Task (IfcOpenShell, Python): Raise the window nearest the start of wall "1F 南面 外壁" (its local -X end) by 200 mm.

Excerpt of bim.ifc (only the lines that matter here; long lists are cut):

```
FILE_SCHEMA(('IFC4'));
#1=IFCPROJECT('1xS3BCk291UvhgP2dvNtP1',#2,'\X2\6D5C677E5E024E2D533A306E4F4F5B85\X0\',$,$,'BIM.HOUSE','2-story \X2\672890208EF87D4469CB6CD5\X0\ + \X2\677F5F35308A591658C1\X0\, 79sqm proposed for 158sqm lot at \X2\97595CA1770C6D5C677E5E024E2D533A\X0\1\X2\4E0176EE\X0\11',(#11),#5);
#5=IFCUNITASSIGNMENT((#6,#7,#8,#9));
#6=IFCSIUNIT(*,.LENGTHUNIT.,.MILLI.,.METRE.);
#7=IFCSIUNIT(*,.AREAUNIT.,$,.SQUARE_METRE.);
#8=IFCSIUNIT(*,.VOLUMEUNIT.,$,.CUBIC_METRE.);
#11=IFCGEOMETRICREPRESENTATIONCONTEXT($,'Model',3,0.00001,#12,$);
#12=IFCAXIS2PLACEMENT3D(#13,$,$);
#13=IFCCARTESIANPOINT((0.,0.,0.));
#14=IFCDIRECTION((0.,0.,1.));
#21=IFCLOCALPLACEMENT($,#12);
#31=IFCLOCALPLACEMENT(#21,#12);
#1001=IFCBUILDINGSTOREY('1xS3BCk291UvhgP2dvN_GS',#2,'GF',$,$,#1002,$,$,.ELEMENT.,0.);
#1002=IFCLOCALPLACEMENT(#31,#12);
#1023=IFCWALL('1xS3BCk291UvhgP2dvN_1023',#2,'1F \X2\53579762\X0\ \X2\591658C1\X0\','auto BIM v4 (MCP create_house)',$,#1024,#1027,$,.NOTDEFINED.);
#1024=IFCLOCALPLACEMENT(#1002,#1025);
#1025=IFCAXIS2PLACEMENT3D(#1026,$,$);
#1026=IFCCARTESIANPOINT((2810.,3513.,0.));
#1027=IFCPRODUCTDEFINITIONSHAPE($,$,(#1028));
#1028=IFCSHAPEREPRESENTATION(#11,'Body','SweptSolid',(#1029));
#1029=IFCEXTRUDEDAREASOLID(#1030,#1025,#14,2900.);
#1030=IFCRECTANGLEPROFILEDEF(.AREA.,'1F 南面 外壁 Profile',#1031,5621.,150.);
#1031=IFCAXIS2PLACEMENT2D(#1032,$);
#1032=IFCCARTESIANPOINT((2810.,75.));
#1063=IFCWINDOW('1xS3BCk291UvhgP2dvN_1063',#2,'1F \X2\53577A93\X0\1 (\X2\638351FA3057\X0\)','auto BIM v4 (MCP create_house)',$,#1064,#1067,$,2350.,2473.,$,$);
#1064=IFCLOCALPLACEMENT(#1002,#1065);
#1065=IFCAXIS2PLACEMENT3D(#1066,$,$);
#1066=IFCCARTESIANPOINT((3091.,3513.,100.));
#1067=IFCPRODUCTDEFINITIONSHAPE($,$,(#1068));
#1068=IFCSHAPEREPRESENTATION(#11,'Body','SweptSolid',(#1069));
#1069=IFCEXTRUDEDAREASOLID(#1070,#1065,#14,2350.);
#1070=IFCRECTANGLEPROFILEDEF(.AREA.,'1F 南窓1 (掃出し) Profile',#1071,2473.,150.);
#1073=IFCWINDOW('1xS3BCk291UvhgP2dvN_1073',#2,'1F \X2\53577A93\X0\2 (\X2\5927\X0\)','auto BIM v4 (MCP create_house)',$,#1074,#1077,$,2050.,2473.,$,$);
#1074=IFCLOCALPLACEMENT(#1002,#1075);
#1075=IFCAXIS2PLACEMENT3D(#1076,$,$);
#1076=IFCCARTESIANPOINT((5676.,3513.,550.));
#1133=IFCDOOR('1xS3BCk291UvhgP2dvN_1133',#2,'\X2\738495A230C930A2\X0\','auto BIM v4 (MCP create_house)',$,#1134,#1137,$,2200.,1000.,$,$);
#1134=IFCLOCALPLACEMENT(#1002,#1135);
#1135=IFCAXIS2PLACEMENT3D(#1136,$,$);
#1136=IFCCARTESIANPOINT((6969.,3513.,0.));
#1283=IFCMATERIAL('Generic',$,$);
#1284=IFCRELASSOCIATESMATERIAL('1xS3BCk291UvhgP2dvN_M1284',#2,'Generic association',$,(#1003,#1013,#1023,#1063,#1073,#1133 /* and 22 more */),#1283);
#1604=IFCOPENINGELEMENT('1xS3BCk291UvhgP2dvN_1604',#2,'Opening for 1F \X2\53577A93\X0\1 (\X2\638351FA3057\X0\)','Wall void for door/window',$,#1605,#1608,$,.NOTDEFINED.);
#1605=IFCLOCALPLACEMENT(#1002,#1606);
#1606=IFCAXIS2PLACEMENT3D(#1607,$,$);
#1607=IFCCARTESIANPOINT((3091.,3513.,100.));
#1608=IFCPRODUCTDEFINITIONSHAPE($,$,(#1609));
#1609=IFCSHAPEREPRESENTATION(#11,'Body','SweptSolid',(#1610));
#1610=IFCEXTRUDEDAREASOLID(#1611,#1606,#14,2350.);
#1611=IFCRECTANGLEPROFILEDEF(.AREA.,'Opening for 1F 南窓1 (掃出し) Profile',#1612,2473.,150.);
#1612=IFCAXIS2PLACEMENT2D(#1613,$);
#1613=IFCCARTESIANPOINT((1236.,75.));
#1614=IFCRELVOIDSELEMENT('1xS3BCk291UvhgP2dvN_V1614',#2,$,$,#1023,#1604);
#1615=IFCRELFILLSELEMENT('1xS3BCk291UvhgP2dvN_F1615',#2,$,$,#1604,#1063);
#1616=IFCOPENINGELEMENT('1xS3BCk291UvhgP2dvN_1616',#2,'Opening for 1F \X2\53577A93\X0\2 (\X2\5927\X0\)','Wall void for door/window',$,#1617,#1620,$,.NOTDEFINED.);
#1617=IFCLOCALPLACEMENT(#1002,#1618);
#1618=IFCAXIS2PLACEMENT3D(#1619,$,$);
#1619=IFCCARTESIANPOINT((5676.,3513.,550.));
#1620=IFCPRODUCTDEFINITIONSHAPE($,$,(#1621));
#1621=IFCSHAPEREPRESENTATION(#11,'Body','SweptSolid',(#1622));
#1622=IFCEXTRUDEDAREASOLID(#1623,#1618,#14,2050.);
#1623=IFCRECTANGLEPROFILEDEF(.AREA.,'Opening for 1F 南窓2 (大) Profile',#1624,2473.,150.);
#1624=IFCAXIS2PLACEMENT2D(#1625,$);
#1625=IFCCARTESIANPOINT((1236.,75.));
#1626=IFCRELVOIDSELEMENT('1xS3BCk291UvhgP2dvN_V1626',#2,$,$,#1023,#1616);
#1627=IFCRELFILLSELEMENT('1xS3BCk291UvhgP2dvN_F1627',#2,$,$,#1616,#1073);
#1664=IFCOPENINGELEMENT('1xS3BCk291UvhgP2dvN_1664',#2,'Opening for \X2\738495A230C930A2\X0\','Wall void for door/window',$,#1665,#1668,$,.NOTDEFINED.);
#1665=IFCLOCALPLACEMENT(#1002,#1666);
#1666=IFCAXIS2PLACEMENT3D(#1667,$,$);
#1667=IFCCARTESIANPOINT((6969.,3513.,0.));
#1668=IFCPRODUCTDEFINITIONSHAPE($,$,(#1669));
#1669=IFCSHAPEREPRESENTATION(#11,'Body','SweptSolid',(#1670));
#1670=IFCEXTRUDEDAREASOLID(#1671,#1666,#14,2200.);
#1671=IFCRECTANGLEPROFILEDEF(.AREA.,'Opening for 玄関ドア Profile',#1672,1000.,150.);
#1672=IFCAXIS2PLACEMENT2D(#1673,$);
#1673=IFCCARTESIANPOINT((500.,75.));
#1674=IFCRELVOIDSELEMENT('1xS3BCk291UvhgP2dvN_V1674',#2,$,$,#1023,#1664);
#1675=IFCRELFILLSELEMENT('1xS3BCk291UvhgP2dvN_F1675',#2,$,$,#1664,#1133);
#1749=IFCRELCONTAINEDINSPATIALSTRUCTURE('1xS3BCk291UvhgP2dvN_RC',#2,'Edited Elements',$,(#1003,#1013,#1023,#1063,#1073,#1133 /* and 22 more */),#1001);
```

```python
import numpy as np
import ifcopenshell
import ifcopenshell.api.geometry
import ifcopenshell.util.placement
import ifcopenshell.util.unit

model = ifcopenshell.open("bim.ifc")
unit_scale = ifcopenshell.util.unit.calculate_unit_scale(model)

window = model.by_guid("1xS3BCk291UvhgP2dvN_1063")
opening = window.FillsVoids[0].RelatingOpeningElement
dz = 0.2 / unit_scale

shift = np.array([0.0, 0.0, dz])
# The window is not placed relative to its opening, so move both.
for product in (opening, window):
    matrix = ifcopenshell.util.placement.get_local_placement(product.ObjectPlacement)
    matrix[:3, 3] += shift
    ifcopenshell.api.geometry.edit_object_placement(model, product=product, matrix=matrix, is_si=False)

print(f"moved by {dz * unit_scale:+.3f} m")

model.write("bim_edited.ifc")
```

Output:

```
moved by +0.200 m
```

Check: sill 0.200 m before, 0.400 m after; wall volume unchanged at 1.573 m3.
